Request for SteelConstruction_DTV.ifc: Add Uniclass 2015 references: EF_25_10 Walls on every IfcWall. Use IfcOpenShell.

First a look at what the model holds.

```python
import ifcopenshell

model = ifcopenshell.open("SteelConstruction_DTV.ifc")
print(model.schema)
print("classifications:", [c.Name for c in model.by_type("IfcClassification")])
for ifc_class in ("IfcDoor", "IfcRoof", "IfcStair", "IfcWall", "IfcWindow"):
    print(ifc_class, len(model.by_type(ifc_class)))
```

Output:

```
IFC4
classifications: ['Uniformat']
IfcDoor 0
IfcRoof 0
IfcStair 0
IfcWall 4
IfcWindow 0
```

```python
import ifcopenshell
import ifcopenshell.api.classification

model = ifcopenshell.open("SteelConstruction_DTV.ifc")

system = ifcopenshell.api.classification.add_classification(model, classification="Uniclass 2015")

codes = {
    "IfcWall": ("EF_25_10", "Walls"),
}
for ifc_class, (code, name) in codes.items():
    products = model.by_type(ifc_class)
    ifcopenshell.api.classification.add_reference(
        model, products=products, classification=system, identification=code, name=name
    )
    print(code, len(products))

model.write("SteelConstruction_DTV_edited.ifc")
```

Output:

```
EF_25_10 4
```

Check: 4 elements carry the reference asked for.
